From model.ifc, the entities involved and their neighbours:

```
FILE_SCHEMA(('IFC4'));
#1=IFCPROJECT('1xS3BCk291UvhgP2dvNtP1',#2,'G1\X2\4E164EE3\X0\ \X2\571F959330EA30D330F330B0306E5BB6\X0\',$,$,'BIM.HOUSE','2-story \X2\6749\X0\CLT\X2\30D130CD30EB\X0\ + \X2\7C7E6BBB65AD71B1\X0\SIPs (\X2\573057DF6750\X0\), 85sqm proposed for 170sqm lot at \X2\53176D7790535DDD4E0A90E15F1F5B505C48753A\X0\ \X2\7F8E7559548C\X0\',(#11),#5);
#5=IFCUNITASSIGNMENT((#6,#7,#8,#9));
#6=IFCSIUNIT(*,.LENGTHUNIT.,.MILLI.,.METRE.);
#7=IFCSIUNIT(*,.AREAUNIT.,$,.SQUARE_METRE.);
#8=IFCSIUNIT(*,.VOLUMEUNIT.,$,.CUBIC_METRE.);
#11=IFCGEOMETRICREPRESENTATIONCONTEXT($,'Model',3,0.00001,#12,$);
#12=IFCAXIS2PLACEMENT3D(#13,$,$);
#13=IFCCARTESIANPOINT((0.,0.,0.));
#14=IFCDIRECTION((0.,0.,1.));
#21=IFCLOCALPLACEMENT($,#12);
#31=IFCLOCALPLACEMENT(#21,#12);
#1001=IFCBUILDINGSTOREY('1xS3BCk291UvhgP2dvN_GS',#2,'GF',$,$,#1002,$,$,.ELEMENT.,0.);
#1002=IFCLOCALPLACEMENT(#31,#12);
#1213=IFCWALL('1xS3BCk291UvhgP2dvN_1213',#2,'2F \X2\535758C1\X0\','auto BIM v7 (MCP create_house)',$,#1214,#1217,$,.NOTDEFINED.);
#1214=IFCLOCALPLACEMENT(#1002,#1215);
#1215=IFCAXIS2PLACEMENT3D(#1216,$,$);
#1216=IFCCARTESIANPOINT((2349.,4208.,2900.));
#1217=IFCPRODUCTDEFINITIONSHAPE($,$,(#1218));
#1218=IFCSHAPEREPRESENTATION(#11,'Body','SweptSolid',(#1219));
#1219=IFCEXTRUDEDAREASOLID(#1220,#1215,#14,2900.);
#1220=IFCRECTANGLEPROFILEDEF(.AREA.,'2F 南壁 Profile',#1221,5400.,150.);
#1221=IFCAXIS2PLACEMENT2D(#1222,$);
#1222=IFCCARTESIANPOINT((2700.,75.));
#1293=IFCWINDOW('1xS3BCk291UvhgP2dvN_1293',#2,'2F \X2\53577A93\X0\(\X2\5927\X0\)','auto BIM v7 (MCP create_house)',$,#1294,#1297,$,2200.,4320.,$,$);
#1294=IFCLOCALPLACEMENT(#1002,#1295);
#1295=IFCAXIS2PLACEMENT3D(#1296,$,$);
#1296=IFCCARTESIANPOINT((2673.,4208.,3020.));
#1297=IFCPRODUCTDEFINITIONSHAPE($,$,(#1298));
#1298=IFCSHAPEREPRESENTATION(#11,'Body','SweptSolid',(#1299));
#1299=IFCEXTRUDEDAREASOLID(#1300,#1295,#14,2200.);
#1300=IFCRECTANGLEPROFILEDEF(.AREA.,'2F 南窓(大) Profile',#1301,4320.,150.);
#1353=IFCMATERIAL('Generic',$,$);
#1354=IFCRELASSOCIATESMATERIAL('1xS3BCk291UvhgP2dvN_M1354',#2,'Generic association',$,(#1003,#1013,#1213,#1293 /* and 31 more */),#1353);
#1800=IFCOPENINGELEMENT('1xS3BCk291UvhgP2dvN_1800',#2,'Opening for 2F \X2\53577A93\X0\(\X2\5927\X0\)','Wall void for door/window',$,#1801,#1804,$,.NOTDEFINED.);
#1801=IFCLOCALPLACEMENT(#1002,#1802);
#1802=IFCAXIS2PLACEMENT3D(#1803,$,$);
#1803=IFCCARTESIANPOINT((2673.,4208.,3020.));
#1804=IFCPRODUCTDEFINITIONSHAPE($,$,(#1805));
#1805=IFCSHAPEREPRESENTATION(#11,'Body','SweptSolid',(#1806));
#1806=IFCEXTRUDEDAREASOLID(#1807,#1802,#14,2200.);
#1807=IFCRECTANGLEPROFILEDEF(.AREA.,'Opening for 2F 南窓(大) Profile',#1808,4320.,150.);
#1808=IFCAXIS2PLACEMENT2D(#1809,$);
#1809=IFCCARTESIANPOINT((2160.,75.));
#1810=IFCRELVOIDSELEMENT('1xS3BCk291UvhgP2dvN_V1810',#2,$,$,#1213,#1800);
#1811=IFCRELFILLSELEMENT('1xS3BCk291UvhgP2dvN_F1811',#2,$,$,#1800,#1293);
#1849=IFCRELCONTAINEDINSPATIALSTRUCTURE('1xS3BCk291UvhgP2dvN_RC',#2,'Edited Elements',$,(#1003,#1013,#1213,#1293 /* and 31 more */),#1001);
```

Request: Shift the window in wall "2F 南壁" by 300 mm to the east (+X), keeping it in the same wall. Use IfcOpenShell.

```python
import ifcopenshell
import ifcopenshell.api.geometry
import ifcopenshell.util.placement
import ifcopenshell.util.unit

model = ifcopenshell.open("model.ifc")
unit_scale = ifcopenshell.util.unit.calculate_unit_scale(model)

window = model.by_guid("1xS3BCk291UvhgP2dvN_1293")
opening = window.FillsVoids[0].RelatingOpeningElement
wall = opening.VoidsElements[0].RelatingBuildingElement

wall_matrix = ifcopenshell.util.placement.get_local_placement(wall.ObjectPlacement)
shift = wall_matrix[:3, 0] * 0.3 / unit_scale
before = ifcopenshell.util.placement.get_local_placement(window.ObjectPlacement)[:3, 3].copy()

# The window is not placed relative to its opening, so move both.
for product in (opening, window):
    matrix = ifcopenshell.util.placement.get_local_placement(product.ObjectPlacement)
    matrix[:3, 3] += shift
    ifcopenshell.api.geometry.edit_object_placement(model, product=product, matrix=matrix, is_si=False)

after = ifcopenshell.util.placement.get_local_placement(window.ObjectPlacement)[:3, 3]
print("window moved by", (after - before).round(3) + 0.0)

model.write("model-out.ifc")
```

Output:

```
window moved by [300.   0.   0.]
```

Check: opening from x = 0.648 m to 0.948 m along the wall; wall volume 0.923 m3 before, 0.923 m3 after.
